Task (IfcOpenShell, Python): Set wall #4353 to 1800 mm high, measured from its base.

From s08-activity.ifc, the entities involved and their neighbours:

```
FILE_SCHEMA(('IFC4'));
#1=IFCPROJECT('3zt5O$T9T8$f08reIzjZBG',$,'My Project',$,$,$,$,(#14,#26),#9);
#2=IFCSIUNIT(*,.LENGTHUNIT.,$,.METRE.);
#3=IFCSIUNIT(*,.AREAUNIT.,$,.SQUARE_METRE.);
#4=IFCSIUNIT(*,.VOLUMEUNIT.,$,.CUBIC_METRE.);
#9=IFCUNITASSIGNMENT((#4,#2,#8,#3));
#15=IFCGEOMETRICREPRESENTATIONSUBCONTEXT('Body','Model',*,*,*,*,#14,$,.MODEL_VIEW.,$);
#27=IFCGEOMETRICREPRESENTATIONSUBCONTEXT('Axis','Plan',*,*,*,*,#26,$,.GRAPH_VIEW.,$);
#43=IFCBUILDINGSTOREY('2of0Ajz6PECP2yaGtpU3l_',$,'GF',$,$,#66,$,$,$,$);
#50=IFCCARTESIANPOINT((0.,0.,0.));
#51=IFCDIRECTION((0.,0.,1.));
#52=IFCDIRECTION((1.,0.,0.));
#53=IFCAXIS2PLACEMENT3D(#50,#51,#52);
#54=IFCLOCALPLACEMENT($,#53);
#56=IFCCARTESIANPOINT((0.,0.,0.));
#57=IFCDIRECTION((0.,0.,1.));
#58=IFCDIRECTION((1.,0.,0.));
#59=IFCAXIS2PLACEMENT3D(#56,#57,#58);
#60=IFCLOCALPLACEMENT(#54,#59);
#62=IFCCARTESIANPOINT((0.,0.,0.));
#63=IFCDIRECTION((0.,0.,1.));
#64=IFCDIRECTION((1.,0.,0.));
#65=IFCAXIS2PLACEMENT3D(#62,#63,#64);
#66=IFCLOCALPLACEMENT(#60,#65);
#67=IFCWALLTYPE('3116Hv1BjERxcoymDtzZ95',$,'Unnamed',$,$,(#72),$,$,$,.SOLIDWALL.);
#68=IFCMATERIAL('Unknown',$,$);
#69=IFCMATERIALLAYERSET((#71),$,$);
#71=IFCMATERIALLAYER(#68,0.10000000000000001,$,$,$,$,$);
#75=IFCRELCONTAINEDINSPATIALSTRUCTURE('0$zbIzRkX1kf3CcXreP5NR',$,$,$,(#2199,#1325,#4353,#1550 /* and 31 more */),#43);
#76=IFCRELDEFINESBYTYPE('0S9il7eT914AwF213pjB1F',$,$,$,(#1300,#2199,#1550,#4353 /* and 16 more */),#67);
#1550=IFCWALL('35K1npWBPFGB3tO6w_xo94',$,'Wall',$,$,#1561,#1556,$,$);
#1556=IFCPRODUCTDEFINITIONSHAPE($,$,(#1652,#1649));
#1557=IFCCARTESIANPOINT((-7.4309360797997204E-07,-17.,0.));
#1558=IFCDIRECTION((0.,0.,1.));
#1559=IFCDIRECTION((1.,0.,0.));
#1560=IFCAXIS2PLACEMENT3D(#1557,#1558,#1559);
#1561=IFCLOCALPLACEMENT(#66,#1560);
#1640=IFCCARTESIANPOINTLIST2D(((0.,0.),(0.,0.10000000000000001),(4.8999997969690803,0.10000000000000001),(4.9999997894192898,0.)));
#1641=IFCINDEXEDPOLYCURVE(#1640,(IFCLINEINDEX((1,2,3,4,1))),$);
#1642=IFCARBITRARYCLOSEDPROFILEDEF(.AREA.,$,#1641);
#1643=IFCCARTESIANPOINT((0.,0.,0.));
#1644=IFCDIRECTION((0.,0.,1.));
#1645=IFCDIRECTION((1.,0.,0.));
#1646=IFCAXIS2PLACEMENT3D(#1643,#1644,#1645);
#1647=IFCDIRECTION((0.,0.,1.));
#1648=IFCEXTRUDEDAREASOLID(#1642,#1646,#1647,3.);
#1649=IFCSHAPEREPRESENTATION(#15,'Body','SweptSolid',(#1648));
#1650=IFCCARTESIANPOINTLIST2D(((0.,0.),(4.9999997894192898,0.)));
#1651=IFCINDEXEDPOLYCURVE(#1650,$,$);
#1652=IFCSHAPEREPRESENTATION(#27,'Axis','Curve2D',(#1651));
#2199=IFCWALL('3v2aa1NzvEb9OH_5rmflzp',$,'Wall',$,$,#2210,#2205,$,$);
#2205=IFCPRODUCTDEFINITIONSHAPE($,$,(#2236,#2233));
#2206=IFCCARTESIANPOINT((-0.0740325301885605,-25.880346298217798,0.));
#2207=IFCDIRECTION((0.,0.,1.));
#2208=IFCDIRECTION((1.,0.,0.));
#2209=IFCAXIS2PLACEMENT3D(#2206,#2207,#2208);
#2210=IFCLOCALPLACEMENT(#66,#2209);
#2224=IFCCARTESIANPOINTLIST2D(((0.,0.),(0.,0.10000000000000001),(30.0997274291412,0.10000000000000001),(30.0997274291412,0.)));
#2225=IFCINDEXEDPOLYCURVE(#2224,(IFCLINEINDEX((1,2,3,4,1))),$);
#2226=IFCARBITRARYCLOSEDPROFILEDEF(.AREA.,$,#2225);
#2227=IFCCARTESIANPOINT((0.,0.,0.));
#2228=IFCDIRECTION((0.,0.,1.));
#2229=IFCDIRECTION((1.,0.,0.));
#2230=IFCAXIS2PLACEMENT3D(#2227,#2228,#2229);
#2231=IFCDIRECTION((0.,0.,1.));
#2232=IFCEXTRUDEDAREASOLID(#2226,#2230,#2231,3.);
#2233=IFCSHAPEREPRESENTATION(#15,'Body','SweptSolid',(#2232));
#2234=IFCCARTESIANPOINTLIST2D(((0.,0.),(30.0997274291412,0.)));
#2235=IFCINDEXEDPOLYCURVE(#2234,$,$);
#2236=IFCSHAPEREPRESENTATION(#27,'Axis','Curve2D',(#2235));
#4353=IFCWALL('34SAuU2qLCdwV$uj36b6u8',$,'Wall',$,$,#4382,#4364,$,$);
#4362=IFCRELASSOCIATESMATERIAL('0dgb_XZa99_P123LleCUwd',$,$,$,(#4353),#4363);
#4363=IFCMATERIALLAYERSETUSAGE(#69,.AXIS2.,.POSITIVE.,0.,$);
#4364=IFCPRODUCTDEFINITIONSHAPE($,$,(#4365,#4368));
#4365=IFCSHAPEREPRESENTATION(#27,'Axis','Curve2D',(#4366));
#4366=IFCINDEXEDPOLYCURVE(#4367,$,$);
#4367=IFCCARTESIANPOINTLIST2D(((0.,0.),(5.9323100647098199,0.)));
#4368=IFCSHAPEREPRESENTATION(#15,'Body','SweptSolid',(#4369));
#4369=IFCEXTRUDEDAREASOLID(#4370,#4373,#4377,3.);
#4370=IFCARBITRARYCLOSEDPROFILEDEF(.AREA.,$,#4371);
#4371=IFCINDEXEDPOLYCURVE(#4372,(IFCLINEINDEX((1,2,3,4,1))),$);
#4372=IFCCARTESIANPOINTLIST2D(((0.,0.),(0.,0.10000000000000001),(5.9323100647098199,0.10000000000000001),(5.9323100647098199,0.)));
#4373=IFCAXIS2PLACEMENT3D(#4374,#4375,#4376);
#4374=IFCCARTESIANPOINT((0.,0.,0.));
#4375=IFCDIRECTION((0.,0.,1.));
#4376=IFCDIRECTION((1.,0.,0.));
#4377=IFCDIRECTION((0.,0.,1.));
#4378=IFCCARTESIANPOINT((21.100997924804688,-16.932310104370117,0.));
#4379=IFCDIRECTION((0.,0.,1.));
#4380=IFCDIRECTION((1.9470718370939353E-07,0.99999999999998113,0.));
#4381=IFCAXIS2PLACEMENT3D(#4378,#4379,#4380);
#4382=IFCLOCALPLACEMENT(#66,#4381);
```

```python
import ifcopenshell
import ifcopenshell.geom
import ifcopenshell.util.representation
import ifcopenshell.util.shape

model = ifcopenshell.open("s08-activity.ifc")
settings = ifcopenshell.geom.settings()


def volume(element):
    """Net volume in cubic metres, openings subtracted."""
    shape = ifcopenshell.geom.create_shape(settings, element)
    return ifcopenshell.util.shape.get_volume(shape.geometry)


wall = model.by_id(4353)
before = volume(wall)

body = ifcopenshell.util.representation.get_representation(wall, "Model", "Body")
solid = body.Items[0]
old_height = solid.Depth
solid.Depth = 1.8
after = volume(wall)

print(f"height {old_height:g} -> {solid.Depth:g}, volume {before:.3f} -> {after:.3f} m3")

model.write("s08-activity_rev.ifc")
```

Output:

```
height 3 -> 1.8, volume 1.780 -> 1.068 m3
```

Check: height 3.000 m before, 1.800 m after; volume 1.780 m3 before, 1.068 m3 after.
